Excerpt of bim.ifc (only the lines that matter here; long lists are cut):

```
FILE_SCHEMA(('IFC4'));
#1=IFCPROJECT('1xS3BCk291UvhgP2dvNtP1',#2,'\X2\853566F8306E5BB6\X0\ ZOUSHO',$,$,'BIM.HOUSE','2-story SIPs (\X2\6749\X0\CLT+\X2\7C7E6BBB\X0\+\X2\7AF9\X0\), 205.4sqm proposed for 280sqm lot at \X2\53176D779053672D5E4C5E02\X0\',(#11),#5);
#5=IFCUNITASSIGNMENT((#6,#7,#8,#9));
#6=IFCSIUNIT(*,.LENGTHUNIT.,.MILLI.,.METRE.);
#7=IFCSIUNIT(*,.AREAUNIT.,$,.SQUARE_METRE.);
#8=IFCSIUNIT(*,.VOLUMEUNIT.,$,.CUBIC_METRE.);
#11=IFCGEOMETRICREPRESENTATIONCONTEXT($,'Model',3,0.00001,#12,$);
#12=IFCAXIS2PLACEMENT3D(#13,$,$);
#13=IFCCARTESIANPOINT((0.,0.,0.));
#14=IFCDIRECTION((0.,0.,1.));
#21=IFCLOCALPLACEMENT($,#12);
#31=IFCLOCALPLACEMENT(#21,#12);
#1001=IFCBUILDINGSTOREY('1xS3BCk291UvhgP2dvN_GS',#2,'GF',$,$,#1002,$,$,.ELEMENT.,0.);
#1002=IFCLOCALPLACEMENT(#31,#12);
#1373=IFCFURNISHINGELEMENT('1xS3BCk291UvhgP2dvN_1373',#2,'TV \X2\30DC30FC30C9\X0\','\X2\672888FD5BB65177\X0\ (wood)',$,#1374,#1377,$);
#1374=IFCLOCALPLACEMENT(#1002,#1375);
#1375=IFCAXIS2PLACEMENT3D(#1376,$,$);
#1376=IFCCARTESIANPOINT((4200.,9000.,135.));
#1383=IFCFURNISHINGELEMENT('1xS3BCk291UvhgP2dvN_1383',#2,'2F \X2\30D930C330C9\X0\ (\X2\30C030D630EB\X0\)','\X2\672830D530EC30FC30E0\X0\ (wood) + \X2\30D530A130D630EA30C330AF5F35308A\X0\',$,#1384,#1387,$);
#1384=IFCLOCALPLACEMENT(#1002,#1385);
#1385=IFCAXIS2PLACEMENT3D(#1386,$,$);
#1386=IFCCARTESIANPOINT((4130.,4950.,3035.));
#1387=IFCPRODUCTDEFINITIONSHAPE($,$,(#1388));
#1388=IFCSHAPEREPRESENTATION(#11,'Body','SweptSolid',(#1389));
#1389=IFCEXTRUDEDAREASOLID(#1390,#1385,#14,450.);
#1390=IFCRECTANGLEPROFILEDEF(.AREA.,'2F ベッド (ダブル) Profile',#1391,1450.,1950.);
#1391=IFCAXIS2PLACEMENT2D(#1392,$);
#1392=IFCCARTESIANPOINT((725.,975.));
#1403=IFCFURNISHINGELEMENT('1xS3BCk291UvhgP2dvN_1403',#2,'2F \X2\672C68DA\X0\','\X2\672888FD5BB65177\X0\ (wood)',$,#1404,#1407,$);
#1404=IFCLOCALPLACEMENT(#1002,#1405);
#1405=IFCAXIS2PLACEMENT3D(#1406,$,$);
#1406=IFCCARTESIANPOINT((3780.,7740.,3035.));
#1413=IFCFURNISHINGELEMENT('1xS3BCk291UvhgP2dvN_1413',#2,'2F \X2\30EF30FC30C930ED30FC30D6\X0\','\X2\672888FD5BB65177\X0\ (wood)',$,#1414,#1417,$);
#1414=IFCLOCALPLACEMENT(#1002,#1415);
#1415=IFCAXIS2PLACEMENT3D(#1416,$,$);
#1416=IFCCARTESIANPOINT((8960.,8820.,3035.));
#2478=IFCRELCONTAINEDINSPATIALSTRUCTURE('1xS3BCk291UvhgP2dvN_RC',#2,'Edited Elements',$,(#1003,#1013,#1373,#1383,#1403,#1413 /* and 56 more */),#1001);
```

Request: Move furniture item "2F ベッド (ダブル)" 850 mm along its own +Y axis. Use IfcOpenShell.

```python
import ifcopenshell
import ifcopenshell.api.geometry
import ifcopenshell.util.placement
import ifcopenshell.util.unit

model = ifcopenshell.open("bim.ifc")
unit_scale = ifcopenshell.util.unit.calculate_unit_scale(model)

item = model.by_guid("1xS3BCk291UvhgP2dvN_1383")
matrix = ifcopenshell.util.placement.get_local_placement(item.ObjectPlacement)
matrix[:3, 3] += matrix[:3, 1] * 0.85 / unit_scale
ifcopenshell.api.geometry.edit_object_placement(model, product=item, matrix=matrix, is_si=False)

print(ifcopenshell.util.placement.get_local_placement(item.ObjectPlacement).round(3) + 0.0)

model.write("bim_updated.ifc")
```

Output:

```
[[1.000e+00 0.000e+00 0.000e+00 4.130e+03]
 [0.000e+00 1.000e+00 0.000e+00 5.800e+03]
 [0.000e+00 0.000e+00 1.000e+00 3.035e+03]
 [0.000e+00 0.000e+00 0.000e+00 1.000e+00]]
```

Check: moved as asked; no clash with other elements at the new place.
